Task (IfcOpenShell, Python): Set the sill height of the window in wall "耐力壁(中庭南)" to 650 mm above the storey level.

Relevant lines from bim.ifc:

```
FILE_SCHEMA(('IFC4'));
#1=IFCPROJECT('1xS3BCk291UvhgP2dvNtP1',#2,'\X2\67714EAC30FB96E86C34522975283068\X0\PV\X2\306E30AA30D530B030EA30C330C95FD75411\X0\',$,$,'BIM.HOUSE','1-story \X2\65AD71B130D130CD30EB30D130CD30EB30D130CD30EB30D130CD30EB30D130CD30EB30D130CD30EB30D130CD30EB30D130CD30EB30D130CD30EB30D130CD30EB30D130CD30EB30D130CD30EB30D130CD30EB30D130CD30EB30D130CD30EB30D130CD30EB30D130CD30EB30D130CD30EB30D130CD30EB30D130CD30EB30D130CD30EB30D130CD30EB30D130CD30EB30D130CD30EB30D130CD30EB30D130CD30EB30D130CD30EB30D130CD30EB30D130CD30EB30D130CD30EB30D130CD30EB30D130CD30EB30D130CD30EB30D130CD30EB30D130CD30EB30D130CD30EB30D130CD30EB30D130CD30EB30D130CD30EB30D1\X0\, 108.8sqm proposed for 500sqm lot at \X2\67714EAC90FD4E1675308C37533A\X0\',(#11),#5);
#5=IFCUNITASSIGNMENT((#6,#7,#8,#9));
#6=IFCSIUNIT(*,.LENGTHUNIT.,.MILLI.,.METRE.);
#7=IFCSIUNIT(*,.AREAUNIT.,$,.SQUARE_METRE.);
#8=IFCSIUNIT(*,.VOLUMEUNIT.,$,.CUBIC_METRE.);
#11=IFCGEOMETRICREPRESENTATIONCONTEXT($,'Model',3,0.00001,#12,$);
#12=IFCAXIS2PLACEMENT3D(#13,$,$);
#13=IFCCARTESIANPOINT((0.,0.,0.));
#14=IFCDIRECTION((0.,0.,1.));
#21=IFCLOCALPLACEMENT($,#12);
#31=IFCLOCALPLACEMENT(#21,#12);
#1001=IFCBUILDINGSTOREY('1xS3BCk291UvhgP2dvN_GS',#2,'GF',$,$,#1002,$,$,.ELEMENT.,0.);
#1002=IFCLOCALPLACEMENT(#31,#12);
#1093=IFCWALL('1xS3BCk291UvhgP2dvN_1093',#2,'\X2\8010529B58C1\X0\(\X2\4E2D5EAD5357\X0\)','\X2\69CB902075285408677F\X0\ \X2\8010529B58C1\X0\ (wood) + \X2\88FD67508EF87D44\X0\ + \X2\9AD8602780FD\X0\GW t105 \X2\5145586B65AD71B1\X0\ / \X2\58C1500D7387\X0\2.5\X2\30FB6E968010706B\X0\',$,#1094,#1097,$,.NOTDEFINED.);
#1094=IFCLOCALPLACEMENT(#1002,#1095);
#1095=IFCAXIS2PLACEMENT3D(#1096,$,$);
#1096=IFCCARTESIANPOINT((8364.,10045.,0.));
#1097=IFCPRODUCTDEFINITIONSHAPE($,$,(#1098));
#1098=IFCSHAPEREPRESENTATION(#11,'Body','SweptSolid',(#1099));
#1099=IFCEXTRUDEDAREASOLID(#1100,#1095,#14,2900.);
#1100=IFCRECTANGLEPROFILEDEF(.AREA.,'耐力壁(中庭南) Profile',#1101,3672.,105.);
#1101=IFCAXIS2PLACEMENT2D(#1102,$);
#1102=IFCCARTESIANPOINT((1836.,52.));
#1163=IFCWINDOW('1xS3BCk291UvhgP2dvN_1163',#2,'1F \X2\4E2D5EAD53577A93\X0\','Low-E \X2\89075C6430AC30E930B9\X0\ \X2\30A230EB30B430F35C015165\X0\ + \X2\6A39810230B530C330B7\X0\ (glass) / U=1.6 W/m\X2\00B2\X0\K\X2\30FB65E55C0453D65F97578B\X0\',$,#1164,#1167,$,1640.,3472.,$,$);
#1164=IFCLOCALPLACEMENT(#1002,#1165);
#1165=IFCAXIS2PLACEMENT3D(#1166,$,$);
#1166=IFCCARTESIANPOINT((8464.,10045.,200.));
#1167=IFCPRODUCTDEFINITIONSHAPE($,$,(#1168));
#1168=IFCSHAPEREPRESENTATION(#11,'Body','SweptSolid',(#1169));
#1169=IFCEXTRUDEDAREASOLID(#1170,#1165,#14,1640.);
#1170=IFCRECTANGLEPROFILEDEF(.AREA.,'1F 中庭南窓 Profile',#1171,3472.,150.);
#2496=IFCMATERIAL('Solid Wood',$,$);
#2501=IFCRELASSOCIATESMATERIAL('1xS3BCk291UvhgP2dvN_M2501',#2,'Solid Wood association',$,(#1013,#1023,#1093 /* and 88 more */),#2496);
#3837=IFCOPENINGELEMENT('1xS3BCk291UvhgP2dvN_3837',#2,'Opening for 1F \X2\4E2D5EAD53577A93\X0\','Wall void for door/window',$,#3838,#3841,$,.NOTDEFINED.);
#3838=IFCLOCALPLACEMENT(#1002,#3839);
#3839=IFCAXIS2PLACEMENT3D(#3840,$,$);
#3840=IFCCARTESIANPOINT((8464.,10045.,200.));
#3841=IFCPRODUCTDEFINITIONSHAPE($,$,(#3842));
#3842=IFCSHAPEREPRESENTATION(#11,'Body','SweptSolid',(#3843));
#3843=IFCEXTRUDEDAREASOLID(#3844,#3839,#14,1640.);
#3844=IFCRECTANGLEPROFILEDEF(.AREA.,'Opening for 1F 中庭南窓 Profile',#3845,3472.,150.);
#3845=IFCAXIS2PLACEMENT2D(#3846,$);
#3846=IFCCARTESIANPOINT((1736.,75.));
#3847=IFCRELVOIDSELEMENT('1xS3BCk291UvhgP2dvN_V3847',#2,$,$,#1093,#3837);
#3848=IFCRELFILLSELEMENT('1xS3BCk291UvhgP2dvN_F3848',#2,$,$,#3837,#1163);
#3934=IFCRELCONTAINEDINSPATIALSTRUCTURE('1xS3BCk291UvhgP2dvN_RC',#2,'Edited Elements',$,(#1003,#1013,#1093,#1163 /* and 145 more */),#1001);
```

```python
import numpy as np
import ifcopenshell
import ifcopenshell.api.geometry
import ifcopenshell.geom
import ifcopenshell.util.element
import ifcopenshell.util.placement
import ifcopenshell.util.shape
import ifcopenshell.util.unit

model = ifcopenshell.open("bim.ifc")
unit_scale = ifcopenshell.util.unit.calculate_unit_scale(model)

window = model.by_guid("1xS3BCk291UvhgP2dvN_1163")
opening = window.FillsVoids[0].RelatingOpeningElement
storey = ifcopenshell.util.element.get_container(window, ifc_class="IfcBuildingStorey")
level = ifcopenshell.util.placement.get_local_placement(storey.ObjectPlacement)[2, 3]

# The opening's origin need not be at the sill, so measure its lowest point.
shape = ifcopenshell.geom.create_shape(ifcopenshell.geom.settings(), opening)
bottom = ifcopenshell.util.shape.get_shape_bottom_elevation(shape, shape.geometry) / unit_scale
dz = level + 650.0 - bottom

shift = np.array([0.0, 0.0, dz])
# The window is not placed relative to its opening, so move both.
for product in (opening, window):
    matrix = ifcopenshell.util.placement.get_local_placement(product.ObjectPlacement)
    matrix[:3, 3] += shift
    ifcopenshell.api.geometry.edit_object_placement(model, product=product, matrix=matrix, is_si=False)

print(f"moved by {dz * unit_scale:+.3f} m")

model.write("bim-out.ifc")
```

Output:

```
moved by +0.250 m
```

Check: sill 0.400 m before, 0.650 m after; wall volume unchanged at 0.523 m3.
